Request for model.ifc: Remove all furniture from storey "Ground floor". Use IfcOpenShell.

First a look at what the model holds.

```python
import ifcopenshell
import ifcopenshell.util.element

model = ifcopenshell.open("model.ifc")
print(model.schema)
storey = next(s for s in model.by_type("IfcBuildingStorey") if s.Name == "Ground floor")
furniture = [e for e in ifcopenshell.util.element.get_decomposition(storey) if e.is_a("IfcFurnishingElement")]
seen = {}
for e in furniture:
    element_type = ifcopenshell.util.element.get_type(e)
    name = element_type.Name if element_type not in (None, e) else None
    seen[name] = seen.get(name, 0) + 1
for name, count in sorted(seen.items(), key=str):
    print(count, "x", name)
```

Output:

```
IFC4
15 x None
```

```python
import ifcopenshell
import ifcopenshell.api.root
import ifcopenshell.util.element

model = ifcopenshell.open("model.ifc")

storey = next(s for s in model.by_type("IfcBuildingStorey") if s.Name == "Ground floor")
furniture = [e for e in ifcopenshell.util.element.get_decomposition(storey) if e.is_a("IfcFurnishingElement")]

for e in furniture:
    ifcopenshell.api.root.remove_product(model, product=e)
print(len(furniture), "removed")

model.write("model_rev.ifc")
```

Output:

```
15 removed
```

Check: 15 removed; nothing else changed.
